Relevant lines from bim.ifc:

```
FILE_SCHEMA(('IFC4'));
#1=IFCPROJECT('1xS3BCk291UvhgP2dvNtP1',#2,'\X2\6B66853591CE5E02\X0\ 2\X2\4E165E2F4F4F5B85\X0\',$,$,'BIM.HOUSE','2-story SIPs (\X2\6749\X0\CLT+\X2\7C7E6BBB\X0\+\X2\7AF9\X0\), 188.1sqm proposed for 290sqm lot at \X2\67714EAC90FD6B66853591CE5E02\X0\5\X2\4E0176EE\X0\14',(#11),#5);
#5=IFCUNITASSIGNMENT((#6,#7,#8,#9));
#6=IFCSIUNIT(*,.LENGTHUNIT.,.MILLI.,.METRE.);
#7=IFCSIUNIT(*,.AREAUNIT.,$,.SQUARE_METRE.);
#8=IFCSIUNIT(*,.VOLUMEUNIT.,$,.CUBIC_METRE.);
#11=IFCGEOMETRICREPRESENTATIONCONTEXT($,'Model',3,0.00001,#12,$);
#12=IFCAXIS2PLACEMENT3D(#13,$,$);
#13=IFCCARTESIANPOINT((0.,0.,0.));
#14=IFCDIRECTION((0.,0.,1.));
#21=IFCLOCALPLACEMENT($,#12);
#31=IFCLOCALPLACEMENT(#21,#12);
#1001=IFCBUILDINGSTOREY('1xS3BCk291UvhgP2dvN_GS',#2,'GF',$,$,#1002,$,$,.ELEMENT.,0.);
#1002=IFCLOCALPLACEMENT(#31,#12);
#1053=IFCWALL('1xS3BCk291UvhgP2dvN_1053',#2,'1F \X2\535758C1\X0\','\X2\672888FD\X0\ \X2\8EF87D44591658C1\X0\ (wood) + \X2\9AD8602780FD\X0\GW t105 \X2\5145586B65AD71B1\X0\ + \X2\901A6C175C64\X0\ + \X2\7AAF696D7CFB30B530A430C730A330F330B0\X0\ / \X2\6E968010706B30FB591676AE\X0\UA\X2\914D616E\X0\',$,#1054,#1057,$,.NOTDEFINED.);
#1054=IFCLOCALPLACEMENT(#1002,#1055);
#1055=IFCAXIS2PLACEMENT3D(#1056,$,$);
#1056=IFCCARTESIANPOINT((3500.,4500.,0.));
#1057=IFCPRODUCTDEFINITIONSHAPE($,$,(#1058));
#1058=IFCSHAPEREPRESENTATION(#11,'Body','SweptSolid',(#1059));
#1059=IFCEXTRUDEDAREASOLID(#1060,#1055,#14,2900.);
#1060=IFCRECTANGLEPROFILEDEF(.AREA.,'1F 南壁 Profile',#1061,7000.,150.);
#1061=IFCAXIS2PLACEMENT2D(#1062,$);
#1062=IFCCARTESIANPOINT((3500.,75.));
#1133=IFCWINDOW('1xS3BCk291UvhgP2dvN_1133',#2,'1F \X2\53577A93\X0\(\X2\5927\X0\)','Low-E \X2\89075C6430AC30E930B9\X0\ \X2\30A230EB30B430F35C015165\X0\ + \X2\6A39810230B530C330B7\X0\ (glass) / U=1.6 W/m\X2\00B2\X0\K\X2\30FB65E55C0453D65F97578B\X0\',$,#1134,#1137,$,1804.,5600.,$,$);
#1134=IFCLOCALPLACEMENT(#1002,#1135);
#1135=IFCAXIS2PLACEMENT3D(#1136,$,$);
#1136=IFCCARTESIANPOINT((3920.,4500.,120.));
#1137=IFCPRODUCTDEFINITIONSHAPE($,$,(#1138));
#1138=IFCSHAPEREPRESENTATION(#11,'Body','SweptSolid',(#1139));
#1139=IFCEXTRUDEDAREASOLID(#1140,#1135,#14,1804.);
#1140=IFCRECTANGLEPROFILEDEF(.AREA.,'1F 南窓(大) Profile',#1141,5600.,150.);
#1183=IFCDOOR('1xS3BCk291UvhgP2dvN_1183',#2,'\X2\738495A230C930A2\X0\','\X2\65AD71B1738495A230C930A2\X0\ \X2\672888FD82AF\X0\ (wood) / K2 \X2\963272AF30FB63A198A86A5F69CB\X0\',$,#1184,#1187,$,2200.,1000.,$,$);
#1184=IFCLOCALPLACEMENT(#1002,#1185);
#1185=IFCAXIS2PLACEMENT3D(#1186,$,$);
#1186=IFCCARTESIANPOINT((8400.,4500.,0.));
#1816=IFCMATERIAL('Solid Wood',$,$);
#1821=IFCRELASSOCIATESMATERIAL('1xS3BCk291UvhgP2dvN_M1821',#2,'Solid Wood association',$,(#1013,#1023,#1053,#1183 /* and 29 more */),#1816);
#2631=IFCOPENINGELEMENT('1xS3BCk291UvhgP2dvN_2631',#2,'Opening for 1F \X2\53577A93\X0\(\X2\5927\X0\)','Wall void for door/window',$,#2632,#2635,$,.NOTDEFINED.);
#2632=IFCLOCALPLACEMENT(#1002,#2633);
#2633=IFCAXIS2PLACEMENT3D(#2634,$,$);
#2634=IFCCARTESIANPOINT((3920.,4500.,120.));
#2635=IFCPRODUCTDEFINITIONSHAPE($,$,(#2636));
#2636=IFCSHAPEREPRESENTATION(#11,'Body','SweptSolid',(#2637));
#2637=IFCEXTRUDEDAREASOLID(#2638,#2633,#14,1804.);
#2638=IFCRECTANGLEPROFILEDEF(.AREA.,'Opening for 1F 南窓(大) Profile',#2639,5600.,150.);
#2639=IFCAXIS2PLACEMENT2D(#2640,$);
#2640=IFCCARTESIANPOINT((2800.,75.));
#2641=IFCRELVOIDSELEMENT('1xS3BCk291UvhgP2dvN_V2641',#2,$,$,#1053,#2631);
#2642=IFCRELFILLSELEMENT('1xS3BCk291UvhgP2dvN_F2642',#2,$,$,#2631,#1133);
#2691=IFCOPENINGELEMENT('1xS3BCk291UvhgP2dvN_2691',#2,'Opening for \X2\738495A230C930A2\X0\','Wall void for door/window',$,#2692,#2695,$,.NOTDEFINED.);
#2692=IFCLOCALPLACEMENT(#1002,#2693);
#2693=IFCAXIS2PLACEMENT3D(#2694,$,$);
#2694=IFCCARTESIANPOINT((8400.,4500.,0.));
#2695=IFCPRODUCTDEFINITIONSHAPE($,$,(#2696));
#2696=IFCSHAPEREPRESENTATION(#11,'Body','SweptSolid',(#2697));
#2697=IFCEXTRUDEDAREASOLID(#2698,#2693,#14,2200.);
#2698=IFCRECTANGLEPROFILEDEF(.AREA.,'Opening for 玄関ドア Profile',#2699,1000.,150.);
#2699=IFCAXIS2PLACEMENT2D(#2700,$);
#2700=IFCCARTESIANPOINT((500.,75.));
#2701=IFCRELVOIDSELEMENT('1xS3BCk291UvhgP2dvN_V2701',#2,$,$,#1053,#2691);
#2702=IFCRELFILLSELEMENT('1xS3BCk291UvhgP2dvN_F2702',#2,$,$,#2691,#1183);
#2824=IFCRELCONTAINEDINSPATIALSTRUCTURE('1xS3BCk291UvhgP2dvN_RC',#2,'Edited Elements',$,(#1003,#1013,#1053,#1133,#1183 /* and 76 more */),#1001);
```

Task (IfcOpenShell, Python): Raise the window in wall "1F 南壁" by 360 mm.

```python
import numpy as np
import ifcopenshell
import ifcopenshell.api.geometry
import ifcopenshell.util.placement
import ifcopenshell.util.unit

model = ifcopenshell.open("bim.ifc")
unit_scale = ifcopenshell.util.unit.calculate_unit_scale(model)

window = model.by_guid("1xS3BCk291UvhgP2dvN_1133")
opening = window.FillsVoids[0].RelatingOpeningElement
dz = 0.36 / unit_scale

shift = np.array([0.0, 0.0, dz])
# The window is not placed relative to its opening, so move both.
for product in (opening, window):
    matrix = ifcopenshell.util.placement.get_local_placement(product.ObjectPlacement)
    matrix[:3, 3] += shift
    ifcopenshell.api.geometry.edit_object_placement(model, product=product, matrix=matrix, is_si=False)

print(f"moved by {dz * unit_scale:+.3f} m")

model.write("bim-out.ifc")
```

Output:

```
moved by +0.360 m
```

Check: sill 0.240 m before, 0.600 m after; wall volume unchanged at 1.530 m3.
